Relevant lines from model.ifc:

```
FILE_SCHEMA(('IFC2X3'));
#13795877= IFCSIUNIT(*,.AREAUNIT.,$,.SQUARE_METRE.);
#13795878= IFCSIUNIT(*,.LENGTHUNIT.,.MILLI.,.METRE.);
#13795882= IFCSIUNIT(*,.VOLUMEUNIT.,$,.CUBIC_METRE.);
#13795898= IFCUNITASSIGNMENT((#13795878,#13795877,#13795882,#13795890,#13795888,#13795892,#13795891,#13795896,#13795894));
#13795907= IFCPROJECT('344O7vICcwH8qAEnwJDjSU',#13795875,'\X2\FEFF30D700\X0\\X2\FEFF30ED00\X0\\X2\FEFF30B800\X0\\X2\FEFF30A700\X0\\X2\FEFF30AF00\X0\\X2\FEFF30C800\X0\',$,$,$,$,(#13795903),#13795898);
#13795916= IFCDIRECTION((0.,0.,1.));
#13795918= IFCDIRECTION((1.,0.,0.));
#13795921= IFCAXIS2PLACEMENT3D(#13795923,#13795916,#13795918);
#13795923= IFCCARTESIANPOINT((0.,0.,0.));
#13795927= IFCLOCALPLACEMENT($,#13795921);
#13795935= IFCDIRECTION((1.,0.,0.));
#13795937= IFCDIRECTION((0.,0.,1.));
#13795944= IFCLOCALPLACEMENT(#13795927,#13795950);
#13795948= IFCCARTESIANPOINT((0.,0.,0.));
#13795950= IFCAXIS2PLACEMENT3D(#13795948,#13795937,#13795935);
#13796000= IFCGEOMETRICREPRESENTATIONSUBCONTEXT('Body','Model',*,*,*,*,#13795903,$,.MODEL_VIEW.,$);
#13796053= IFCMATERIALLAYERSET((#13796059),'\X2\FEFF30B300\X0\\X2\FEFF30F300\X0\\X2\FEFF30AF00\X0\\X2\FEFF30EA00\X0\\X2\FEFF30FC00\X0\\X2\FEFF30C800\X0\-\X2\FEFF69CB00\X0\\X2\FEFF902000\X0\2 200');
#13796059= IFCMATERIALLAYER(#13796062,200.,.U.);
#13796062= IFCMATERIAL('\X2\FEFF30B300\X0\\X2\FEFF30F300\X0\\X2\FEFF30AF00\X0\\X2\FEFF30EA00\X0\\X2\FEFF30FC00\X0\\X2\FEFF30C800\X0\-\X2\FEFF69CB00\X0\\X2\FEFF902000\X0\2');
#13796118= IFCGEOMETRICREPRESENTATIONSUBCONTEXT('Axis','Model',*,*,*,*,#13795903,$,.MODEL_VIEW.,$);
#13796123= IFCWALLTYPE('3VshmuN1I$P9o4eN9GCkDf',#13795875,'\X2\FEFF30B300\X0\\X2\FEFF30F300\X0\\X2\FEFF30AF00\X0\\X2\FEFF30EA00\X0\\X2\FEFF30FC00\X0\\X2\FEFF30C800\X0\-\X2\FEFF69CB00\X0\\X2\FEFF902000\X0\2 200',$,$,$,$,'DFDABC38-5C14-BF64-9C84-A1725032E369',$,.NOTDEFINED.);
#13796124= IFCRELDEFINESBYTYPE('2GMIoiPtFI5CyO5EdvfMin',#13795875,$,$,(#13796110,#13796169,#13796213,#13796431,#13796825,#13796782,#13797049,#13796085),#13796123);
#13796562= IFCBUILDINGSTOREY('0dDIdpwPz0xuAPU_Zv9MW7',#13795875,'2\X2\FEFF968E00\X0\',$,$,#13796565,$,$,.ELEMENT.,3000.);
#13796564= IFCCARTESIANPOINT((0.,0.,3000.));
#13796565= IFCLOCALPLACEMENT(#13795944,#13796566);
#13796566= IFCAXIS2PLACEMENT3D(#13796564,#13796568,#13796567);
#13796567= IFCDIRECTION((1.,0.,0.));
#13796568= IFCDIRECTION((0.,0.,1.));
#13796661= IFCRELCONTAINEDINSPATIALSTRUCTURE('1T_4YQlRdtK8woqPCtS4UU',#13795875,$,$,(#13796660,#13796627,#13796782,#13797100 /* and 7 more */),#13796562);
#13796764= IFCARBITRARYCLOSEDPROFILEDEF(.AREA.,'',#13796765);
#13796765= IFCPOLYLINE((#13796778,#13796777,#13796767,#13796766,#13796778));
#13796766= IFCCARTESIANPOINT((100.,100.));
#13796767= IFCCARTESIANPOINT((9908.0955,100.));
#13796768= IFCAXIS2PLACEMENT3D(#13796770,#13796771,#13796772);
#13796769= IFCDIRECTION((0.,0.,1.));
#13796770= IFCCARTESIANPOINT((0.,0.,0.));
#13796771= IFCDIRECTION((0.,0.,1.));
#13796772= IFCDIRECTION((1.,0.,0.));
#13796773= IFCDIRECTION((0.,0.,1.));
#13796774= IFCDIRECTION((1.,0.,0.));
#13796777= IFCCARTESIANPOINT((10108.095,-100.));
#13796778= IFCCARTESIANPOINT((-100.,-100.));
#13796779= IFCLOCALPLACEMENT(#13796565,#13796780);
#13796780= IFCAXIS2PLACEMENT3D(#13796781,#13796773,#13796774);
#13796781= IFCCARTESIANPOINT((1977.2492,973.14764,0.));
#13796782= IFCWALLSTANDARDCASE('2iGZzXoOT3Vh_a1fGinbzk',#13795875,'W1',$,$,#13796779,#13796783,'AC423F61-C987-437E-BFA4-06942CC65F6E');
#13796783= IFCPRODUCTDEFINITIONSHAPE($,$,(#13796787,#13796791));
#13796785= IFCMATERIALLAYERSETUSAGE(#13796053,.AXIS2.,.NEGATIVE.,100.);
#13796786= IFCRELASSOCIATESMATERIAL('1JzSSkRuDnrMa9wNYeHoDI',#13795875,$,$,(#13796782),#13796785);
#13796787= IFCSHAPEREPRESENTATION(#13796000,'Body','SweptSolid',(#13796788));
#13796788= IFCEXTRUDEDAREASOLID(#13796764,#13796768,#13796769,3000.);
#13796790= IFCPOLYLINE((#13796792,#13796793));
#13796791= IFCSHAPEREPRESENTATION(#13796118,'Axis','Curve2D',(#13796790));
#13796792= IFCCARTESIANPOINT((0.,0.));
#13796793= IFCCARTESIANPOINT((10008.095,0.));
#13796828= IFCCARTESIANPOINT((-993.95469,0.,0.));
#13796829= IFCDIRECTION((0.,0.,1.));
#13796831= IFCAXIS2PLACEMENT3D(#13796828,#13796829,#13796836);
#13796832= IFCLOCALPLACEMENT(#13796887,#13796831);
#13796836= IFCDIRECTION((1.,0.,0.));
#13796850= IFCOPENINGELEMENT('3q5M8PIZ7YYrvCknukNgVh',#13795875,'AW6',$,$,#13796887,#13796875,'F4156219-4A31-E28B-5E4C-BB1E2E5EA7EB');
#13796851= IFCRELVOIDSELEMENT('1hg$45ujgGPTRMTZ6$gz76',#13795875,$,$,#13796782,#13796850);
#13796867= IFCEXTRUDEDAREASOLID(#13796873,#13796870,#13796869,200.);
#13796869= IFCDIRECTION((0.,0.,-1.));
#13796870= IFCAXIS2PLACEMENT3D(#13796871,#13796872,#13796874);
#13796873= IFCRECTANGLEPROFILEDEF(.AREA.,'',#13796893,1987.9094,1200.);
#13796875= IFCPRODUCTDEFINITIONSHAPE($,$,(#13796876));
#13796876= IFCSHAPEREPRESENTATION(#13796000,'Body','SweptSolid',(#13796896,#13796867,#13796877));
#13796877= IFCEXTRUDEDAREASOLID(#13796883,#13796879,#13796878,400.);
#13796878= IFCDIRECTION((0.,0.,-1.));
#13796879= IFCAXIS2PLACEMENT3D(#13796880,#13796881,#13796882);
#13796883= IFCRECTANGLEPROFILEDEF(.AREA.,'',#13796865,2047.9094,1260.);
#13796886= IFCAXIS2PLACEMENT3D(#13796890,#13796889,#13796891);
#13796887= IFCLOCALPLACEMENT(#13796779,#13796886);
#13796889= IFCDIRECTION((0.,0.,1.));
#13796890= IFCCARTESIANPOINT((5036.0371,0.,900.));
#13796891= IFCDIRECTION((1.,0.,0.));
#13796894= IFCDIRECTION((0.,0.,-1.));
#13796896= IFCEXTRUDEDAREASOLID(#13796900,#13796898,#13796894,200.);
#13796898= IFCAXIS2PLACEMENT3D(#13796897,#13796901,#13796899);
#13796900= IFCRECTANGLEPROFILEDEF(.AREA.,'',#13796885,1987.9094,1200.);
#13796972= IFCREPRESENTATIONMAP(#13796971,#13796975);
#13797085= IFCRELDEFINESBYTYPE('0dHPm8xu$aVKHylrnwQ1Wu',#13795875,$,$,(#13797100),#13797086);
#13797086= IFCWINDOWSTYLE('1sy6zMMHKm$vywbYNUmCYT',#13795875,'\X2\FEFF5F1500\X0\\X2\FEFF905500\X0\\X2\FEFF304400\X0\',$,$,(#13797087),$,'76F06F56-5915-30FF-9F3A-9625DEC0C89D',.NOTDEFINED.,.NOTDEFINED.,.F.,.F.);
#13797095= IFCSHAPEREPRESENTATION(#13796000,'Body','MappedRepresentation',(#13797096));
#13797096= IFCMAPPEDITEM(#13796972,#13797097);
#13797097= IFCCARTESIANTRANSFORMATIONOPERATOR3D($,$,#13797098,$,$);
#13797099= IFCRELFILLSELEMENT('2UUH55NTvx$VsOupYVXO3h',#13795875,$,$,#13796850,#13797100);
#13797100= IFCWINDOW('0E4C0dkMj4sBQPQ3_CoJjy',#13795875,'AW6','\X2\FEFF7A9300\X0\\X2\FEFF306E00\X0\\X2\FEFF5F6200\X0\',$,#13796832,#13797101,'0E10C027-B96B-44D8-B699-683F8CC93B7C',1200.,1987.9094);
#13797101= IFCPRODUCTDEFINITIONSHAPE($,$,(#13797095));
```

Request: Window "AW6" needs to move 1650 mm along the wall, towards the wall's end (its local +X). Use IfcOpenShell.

```python
import ifcopenshell
import ifcopenshell.api.geometry
import ifcopenshell.util.placement

model = ifcopenshell.open("model.ifc")

window = model.by_guid("0E4C0dkMj4sBQPQ3_CoJjy")
opening = window.FillsVoids[0].RelatingOpeningElement
wall = opening.VoidsElements[0].RelatingBuildingElement

wall_matrix = ifcopenshell.util.placement.get_local_placement(wall.ObjectPlacement)
shift = wall_matrix[:3, 0] * 1650.0
before = ifcopenshell.util.placement.get_local_placement(window.ObjectPlacement)[:3, 3].copy()

# The window is placed relative to its opening, so it follows when the opening moves.
matrix = ifcopenshell.util.placement.get_local_placement(opening.ObjectPlacement)
matrix[:3, 3] += shift
ifcopenshell.api.geometry.edit_object_placement(
    model, product=opening, matrix=matrix, is_si=False, should_transform_children=True
)

after = ifcopenshell.util.placement.get_local_placement(window.ObjectPlacement)[:3, 3]
print("window moved by", (after - before).round(3) + 0.0)

model.write("model_rev.ifc")
```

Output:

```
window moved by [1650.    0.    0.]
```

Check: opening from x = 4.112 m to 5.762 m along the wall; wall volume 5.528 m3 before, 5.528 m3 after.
